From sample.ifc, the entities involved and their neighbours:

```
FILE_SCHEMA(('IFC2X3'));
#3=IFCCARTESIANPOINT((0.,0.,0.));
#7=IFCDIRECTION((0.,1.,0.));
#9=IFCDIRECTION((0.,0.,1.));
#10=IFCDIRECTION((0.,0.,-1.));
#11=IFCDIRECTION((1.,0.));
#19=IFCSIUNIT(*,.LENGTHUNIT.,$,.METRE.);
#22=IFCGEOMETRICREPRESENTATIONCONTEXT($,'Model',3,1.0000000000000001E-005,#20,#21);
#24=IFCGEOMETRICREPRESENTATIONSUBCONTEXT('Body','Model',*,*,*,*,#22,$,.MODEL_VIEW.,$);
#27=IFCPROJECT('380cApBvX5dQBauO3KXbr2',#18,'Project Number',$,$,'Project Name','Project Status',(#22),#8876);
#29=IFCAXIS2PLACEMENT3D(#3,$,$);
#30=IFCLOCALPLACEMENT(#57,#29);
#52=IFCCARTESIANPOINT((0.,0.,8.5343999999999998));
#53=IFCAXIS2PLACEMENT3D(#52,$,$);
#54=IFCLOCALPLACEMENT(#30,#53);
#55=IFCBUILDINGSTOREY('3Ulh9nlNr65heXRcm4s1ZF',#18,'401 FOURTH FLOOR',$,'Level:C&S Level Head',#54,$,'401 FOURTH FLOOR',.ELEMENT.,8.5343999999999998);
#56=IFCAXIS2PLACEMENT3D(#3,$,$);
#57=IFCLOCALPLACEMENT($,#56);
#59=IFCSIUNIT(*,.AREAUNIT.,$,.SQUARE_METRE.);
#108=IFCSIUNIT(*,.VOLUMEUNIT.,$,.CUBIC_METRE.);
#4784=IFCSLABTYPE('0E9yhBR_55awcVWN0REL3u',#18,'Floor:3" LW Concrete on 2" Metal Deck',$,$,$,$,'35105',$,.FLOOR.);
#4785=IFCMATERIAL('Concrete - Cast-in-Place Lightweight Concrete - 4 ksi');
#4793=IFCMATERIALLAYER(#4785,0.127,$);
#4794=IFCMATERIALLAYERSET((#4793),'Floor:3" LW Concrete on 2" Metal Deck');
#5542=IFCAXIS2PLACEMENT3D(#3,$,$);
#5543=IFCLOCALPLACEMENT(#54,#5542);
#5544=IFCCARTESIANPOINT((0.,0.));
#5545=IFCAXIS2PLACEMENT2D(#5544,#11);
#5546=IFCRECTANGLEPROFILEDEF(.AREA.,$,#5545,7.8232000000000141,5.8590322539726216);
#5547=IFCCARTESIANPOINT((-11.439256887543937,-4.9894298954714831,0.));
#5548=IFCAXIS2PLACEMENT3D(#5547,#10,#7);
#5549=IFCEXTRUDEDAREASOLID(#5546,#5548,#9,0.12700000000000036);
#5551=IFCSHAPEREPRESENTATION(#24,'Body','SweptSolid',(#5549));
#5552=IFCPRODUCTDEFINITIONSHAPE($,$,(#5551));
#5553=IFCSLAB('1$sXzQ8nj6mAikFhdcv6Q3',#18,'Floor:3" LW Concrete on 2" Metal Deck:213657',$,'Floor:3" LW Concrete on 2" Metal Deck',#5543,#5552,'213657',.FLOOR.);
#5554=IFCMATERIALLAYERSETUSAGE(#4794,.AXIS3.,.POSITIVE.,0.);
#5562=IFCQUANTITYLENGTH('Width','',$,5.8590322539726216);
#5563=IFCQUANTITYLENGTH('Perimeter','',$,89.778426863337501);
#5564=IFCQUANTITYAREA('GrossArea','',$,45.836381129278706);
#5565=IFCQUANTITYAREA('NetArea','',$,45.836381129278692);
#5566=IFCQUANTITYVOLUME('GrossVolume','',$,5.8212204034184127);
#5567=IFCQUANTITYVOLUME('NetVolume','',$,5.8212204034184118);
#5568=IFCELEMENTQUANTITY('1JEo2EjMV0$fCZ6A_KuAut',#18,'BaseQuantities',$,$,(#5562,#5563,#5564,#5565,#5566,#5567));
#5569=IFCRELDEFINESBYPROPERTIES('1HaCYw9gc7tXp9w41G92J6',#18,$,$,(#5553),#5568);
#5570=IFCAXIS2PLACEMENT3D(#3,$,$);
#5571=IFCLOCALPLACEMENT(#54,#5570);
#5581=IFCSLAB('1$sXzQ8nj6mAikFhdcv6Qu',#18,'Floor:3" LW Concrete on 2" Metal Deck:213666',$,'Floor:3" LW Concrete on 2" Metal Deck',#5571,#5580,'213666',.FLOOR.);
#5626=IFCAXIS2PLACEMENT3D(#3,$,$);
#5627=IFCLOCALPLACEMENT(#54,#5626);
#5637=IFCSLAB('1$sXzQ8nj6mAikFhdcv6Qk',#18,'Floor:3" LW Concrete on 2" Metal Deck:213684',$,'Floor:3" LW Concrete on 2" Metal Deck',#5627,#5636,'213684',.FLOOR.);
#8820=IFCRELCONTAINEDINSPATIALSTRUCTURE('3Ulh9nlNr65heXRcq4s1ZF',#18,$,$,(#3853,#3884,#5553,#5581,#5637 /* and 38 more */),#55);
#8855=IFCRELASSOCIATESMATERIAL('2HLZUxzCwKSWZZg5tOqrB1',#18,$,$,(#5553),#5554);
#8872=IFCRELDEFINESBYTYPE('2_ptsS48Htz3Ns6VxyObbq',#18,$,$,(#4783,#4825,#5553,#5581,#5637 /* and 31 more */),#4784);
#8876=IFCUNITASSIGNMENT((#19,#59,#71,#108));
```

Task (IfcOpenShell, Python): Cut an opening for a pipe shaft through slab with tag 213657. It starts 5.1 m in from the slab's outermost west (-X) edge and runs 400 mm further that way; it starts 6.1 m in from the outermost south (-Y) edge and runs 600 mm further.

```python
import numpy as np
import ifcopenshell
import ifcopenshell.api.feature
import ifcopenshell.api.geometry
import ifcopenshell.api.pset
import ifcopenshell.api.root
import ifcopenshell.geom
import ifcopenshell.util.element
import ifcopenshell.util.placement
import ifcopenshell.util.representation
import ifcopenshell.util.shape
import ifcopenshell.util.unit

model = ifcopenshell.open("sample.ifc")
unit_scale = ifcopenshell.util.unit.calculate_unit_scale(model)
area_scale = ifcopenshell.util.unit.calculate_unit_scale(model, "AREAUNIT")
volume_scale = ifcopenshell.util.unit.calculate_unit_scale(model, "VOLUMEUNIT")
settings = ifcopenshell.geom.settings()


def volume(element):
    """Net volume in cubic metres, openings subtracted."""
    shape = ifcopenshell.geom.create_shape(settings, element)
    return ifcopenshell.util.shape.get_volume(shape.geometry)


slab = model.by_guid("1$sXzQ8nj6mAikFhdcv6Q3")
before = volume(slab)

# Extent in the slab's own axes, in metres. The edges named are its -X and -Y sides.
slab_shape = ifcopenshell.geom.create_shape(settings, slab)
vertices = ifcopenshell.util.shape.get_vertices(slab_shape.geometry)
x_min, y_min, bottom = vertices.min(axis=0)
top = vertices[:, 2].max()

opening = ifcopenshell.api.root.create_entity(model, ifc_class="IfcOpeningElement", name="Pipe shaft opening")
context = ifcopenshell.util.representation.get_context(model, "Model", "Body", "MODEL_VIEW")
width, depth = 0.4, 0.6
outline = [(0.0, 0.0), (width, 0.0), (width, depth), (0.0, depth), (0.0, 0.0)]
# Overshoot both faces by 50 mm so the cut is clean.
shape = ifcopenshell.api.geometry.add_slab_representation(
    model, context=context, depth=top - bottom + 0.1, polyline=outline
)
ifcopenshell.api.geometry.assign_representation(model, product=opening, representation=shape)

matrix = ifcopenshell.util.placement.get_local_placement(slab.ObjectPlacement)
matrix[:, 3] = matrix @ np.append(np.array([x_min + 5.1, y_min + 6.1, bottom - 0.05]) / unit_scale, 1.0)
ifcopenshell.api.geometry.edit_object_placement(model, product=opening, matrix=matrix, is_si=False)
ifcopenshell.api.feature.add_feature(model, feature=opening, element=slab)

after = volume(slab)

# Update the slab's stored quantities.
qto = model.by_id(ifcopenshell.util.element.get_pset(slab, "BaseQuantities", should_inherit=False)["id"])
ifcopenshell.api.pset.edit_qto(model, qto=qto, properties={
    "NetArea": after / (top - bottom) / area_scale,
    "NetVolume": after / volume_scale,
})

print(f"slab volume {before:.3f} -> {after:.3f} m3")

model.write("sample_v2.ifc")
```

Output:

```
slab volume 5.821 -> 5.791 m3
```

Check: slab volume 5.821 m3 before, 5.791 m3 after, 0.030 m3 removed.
